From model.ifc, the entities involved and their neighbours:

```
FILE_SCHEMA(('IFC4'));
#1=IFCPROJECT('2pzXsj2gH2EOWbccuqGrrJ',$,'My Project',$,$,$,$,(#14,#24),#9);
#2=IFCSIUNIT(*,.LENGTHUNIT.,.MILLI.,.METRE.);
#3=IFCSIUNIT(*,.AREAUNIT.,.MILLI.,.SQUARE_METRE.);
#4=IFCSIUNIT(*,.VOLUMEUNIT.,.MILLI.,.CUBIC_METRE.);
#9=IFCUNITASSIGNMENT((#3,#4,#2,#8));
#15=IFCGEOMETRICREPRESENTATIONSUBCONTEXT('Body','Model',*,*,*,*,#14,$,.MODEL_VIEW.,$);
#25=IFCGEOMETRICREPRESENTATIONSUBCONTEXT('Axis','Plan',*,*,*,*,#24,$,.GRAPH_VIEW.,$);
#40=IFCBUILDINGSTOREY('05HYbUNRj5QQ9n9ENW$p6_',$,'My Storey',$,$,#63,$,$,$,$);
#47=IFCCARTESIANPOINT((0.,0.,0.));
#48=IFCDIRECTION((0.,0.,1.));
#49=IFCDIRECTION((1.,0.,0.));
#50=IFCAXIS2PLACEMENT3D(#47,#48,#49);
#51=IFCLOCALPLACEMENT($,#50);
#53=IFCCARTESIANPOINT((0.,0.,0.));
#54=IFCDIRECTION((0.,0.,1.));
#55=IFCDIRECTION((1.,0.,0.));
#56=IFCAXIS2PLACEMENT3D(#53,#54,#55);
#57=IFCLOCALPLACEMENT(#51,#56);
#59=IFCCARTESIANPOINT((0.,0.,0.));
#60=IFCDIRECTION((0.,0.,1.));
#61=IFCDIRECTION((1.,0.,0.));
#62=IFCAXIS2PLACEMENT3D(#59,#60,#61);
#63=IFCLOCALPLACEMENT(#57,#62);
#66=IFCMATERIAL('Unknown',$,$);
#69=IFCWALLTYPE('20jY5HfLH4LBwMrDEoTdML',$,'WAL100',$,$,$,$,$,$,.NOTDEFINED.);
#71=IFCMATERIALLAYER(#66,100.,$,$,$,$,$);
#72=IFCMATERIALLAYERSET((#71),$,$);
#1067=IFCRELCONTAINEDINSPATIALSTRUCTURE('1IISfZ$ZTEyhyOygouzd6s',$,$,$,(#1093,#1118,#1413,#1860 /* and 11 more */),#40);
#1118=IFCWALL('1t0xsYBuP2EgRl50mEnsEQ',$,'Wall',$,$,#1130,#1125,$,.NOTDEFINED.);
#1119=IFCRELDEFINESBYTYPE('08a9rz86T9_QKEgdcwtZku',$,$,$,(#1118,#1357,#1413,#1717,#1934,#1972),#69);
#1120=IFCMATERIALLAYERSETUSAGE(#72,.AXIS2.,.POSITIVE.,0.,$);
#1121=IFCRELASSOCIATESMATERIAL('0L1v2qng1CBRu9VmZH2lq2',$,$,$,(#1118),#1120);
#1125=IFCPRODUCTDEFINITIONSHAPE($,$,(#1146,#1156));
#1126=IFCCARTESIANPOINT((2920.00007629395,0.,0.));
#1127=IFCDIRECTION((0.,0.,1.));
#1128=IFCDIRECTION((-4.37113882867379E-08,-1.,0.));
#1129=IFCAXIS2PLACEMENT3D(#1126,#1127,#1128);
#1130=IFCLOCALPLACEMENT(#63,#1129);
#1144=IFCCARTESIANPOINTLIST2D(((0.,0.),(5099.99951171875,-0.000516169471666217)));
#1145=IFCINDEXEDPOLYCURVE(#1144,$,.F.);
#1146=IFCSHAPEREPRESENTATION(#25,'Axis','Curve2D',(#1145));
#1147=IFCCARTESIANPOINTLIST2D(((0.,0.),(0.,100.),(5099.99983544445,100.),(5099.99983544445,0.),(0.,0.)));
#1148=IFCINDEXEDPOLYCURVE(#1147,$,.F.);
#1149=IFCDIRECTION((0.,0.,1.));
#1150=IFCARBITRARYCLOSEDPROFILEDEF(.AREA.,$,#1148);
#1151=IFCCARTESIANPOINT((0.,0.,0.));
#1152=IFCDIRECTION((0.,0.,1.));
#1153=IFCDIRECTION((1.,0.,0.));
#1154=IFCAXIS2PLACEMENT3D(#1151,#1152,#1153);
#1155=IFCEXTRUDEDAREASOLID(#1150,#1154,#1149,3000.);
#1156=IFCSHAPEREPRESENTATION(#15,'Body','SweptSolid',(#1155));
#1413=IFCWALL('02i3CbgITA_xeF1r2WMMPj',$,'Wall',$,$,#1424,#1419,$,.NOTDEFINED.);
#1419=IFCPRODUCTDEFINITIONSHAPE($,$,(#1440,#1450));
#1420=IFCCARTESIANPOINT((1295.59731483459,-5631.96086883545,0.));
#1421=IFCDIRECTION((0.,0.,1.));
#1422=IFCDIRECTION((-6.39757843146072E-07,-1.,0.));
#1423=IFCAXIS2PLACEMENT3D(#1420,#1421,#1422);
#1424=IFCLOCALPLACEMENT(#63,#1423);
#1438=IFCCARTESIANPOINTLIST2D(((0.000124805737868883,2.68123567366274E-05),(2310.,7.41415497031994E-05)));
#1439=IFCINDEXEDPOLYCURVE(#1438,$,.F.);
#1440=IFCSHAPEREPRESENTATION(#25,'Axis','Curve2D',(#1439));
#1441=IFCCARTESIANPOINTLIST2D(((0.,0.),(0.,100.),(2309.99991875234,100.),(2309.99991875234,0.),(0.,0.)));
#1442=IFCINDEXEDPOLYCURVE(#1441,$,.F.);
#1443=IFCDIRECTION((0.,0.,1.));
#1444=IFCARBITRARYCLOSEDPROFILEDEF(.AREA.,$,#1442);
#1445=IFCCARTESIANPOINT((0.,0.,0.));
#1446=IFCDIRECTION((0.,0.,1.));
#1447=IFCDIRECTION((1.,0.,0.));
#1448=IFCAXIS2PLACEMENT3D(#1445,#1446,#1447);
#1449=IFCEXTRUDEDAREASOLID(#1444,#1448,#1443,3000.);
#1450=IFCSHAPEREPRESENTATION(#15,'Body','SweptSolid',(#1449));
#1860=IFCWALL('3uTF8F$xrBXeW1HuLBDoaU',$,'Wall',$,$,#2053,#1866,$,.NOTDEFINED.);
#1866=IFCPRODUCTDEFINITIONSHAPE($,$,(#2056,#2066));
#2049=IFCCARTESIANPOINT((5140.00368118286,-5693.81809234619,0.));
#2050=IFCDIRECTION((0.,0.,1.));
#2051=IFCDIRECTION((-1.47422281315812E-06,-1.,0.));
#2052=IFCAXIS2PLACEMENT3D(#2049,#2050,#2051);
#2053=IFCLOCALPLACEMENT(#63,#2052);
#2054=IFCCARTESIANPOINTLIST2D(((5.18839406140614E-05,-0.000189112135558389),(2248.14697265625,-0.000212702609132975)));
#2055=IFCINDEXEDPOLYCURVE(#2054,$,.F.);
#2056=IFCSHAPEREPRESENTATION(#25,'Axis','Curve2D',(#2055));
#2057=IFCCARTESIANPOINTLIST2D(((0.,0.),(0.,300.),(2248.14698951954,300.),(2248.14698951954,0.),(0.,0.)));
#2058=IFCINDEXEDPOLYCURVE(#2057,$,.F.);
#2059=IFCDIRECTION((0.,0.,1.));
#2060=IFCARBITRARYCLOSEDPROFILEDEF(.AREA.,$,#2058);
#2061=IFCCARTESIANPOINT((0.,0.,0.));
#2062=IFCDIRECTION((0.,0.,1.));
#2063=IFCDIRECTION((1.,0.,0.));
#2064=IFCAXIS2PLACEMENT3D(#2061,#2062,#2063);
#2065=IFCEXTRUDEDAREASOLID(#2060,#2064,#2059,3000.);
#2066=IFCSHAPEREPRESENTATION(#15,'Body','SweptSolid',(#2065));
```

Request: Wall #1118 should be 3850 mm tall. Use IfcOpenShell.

```python
import ifcopenshell
import ifcopenshell.geom
import ifcopenshell.util.representation
import ifcopenshell.util.shape

model = ifcopenshell.open("model.ifc")
settings = ifcopenshell.geom.settings()


def volume(element):
    """Net volume in cubic metres, openings subtracted."""
    shape = ifcopenshell.geom.create_shape(settings, element)
    return ifcopenshell.util.shape.get_volume(shape.geometry)


wall = model.by_id(1118)
before = volume(wall)

body = ifcopenshell.util.representation.get_representation(wall, "Model", "Body")
solid = body.Items[0]
old_height = solid.Depth
solid.Depth = 3850.0
after = volume(wall)

print(f"height {old_height:g} -> {solid.Depth:g}, volume {before:.3f} -> {after:.3f} m3")

model.write("model-out.ifc")
```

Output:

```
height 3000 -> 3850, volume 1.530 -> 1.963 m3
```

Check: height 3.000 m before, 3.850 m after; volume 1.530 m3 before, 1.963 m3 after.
